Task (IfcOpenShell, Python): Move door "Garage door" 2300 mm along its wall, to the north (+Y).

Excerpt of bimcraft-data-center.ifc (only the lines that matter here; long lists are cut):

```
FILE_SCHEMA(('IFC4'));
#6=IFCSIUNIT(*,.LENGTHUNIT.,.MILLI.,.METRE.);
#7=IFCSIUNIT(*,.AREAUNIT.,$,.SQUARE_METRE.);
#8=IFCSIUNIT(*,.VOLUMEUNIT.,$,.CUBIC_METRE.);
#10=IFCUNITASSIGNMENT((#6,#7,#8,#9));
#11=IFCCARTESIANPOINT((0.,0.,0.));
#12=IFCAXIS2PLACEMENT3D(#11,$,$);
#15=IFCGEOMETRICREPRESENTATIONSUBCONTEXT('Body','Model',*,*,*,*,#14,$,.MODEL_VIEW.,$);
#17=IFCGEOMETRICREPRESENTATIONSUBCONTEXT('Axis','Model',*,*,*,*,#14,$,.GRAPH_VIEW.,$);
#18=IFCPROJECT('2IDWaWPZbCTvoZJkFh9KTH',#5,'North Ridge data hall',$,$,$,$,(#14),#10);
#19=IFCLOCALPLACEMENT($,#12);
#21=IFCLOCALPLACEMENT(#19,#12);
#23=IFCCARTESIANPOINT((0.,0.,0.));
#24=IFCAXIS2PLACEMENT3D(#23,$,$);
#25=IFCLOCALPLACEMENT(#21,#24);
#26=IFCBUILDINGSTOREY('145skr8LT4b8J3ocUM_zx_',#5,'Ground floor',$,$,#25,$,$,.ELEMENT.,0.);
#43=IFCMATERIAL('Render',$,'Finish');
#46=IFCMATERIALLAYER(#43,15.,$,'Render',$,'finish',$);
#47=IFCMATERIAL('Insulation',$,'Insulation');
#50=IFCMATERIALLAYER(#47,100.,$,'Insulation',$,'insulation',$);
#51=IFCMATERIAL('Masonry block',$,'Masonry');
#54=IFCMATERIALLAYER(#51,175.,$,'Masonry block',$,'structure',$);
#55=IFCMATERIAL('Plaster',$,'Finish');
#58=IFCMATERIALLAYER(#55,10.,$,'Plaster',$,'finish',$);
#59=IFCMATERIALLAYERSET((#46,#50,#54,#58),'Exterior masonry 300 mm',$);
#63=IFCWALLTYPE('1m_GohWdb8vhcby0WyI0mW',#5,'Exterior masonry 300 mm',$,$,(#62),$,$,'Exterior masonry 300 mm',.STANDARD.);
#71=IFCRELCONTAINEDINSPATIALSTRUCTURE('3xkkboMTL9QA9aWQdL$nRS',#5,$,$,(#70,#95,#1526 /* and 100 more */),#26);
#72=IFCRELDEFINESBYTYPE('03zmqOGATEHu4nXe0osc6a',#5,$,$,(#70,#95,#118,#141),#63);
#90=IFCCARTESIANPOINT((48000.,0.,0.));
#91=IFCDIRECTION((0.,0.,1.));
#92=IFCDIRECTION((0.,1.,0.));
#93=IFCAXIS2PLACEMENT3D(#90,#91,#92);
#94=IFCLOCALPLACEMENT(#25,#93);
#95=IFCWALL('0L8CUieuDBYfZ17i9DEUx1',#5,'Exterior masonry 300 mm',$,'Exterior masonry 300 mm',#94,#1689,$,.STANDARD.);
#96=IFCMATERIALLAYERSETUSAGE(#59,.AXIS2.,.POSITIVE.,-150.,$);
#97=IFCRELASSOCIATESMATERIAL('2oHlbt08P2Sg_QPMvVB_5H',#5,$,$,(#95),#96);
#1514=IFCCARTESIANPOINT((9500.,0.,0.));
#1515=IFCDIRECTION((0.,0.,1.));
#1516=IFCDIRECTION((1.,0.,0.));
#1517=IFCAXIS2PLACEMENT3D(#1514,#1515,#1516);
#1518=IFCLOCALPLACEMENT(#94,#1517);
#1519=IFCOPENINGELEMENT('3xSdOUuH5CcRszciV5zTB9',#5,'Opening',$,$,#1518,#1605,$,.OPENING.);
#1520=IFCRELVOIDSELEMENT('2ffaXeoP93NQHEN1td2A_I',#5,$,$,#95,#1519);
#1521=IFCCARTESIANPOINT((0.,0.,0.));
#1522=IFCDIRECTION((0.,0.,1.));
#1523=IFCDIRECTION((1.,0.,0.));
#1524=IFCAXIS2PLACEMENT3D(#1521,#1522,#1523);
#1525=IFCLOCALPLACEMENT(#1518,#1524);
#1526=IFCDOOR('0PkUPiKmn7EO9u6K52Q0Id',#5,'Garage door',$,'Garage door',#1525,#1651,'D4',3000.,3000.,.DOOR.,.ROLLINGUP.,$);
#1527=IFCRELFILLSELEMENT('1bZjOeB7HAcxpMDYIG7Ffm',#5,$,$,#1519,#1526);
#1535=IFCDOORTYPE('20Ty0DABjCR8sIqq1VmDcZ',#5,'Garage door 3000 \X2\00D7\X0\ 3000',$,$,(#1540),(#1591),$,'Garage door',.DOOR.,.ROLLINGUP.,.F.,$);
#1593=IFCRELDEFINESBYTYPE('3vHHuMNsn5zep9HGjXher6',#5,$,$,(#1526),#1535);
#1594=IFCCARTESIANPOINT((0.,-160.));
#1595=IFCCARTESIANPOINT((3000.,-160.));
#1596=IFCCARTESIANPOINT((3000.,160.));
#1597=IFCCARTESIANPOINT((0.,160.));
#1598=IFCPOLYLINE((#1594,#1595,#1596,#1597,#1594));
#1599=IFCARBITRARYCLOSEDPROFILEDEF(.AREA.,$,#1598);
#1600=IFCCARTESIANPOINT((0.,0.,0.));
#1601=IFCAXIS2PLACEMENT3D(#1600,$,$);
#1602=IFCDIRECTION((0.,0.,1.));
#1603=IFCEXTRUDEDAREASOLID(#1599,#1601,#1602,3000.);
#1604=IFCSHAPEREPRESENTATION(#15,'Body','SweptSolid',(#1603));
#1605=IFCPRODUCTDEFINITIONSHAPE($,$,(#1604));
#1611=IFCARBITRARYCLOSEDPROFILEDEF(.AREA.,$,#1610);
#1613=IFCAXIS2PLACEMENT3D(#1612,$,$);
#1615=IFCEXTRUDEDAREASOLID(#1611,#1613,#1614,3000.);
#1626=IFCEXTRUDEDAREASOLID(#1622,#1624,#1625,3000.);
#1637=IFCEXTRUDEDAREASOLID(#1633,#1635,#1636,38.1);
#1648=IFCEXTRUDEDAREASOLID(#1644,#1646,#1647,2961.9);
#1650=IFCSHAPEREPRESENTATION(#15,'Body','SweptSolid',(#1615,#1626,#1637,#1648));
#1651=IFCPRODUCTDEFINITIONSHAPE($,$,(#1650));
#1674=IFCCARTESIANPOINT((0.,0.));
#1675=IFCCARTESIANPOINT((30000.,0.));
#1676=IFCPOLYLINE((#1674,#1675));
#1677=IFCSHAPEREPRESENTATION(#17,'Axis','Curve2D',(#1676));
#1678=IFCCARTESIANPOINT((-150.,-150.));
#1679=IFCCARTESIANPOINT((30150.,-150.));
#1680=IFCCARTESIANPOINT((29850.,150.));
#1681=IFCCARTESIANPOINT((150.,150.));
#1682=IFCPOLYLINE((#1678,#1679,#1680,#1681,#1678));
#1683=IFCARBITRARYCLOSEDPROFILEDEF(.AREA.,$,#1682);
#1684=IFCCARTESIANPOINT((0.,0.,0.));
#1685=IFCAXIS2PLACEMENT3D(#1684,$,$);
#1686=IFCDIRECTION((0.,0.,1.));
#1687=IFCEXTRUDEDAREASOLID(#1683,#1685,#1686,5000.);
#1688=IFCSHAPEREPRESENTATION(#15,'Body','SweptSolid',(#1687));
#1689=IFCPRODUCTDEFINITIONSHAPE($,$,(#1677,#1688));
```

```python
import ifcopenshell
import ifcopenshell.api.geometry
import ifcopenshell.util.placement

model = ifcopenshell.open("bimcraft-data-center.ifc")

door = model.by_guid("0PkUPiKmn7EO9u6K52Q0Id")
opening = door.FillsVoids[0].RelatingOpeningElement
wall = opening.VoidsElements[0].RelatingBuildingElement

wall_matrix = ifcopenshell.util.placement.get_local_placement(wall.ObjectPlacement)
shift = wall_matrix[:3, 0] * 2300.0
before = ifcopenshell.util.placement.get_local_placement(door.ObjectPlacement)[:3, 3].copy()

# The door is placed relative to its opening, so it follows when the opening moves.
matrix = ifcopenshell.util.placement.get_local_placement(opening.ObjectPlacement)
matrix[:3, 3] += shift
ifcopenshell.api.geometry.edit_object_placement(
    model, product=opening, matrix=matrix, is_si=False, should_transform_children=True
)

after = ifcopenshell.util.placement.get_local_placement(door.ObjectPlacement)[:3, 3]
print("door moved by", (after - before).round(3) + 0.0)

model.write("bimcraft-data-center_v2.ifc")
```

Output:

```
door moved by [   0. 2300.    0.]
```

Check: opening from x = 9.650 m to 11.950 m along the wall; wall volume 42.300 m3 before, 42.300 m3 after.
